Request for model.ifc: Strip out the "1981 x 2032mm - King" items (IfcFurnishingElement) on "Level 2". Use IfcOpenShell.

First a look at what the model holds.

```python
import ifcopenshell
import ifcopenshell.util.element

model = ifcopenshell.open("model.ifc")
print(model.schema)
storey = next(s for s in model.by_type("IfcBuildingStorey") if s.Name == "Level 2")
furniture = [e for e in ifcopenshell.util.element.get_decomposition(storey) if e.is_a("IfcFurnishingElement")]
seen = {}
for e in furniture:
    element_type = ifcopenshell.util.element.get_type(e)
    name = element_type.Name if element_type not in (None, e) else None
    seen[name] = seen.get(name, 0) + 1
for name, count in sorted(seen.items(), key=str):
    print(count, "x", name)
```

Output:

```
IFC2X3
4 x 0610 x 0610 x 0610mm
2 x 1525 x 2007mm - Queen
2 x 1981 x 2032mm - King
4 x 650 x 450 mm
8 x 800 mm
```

```python
import ifcopenshell
import ifcopenshell.api.root
import ifcopenshell.util.element

model = ifcopenshell.open("model.ifc")

storey = next(s for s in model.by_type("IfcBuildingStorey") if s.Name == "Level 2")
furniture = [e for e in ifcopenshell.util.element.get_decomposition(storey) if e.is_a("IfcFurnishingElement")]
targets = [e for e in furniture if (t := ifcopenshell.util.element.get_type(e)) not in (None, e) and t.Name == "1981 x 2032mm - King"]

for e in targets:
    ifcopenshell.api.root.remove_product(model, product=e)
print(len(targets), "removed")

model.write("model_v2.ifc")
```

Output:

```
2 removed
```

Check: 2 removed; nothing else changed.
